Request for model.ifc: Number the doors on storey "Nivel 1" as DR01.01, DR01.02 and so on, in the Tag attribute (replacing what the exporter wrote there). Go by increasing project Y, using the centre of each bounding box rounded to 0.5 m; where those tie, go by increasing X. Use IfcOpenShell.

First a look at what the model holds.

```python
import ifcopenshell
import ifcopenshell.util.element
import ifcopenshell.util.placement

model = ifcopenshell.open("model.ifc")
print(model.schema)
storey = next(s for s in model.by_type("IfcBuildingStorey") if s.Name == "Nivel 1")
doors = [e for e in ifcopenshell.util.element.get_decomposition(storey) if e.is_a("IfcDoor")]
for e in sorted(doors, key=lambda e: e.id()):
    origin = ifcopenshell.util.placement.get_local_placement(e.ObjectPlacement)[:3, 3]
    print(e.id(), e.Tag, e.Name, origin.round(2) + 0.0, sep=" | ")
```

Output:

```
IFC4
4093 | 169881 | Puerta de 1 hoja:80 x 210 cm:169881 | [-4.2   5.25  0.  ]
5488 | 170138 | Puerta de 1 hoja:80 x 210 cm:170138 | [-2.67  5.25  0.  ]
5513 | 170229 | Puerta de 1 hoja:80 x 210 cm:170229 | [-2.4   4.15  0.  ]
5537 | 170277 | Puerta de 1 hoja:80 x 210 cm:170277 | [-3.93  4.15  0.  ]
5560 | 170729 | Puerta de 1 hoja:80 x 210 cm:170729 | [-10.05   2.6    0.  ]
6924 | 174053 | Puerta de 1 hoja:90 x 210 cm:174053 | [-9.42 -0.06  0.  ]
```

```python
import ifcopenshell
import ifcopenshell.geom
import ifcopenshell.util.element
import ifcopenshell.util.shape

model = ifcopenshell.open("model.ifc")
settings = ifcopenshell.geom.settings()
settings.set("use-world-coords", True)


def centre(element):
    shape = ifcopenshell.geom.create_shape(settings, element)
    return ifcopenshell.util.shape.get_bbox_centroid(shape.geometry)


storey = next(s for s in model.by_type("IfcBuildingStorey") if s.Name == "Nivel 1")
doors = [e for e in ifcopenshell.util.element.get_decomposition(storey) if e.is_a("IfcDoor")]

# Insertion points can sit at a corner or the storey origin, so sort by the geometry (in metres).
centres = {e: centre(e) for e in doors}
doors.sort(key=lambda e: (round(centres[e][1] / 0.5), centres[e][0]))

for i, e in enumerate(doors, start=1):
    number = f"DR01.{i:02d}"
    e.Tag = number
    print(e.id(), number)

model.write("model-out.ifc")
```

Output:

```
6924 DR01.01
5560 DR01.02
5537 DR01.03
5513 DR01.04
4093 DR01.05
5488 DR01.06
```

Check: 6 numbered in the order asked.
